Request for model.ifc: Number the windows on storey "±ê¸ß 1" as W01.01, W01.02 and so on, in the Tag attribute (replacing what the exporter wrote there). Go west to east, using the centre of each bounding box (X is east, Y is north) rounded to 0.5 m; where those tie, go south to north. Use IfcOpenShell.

First a look at what the model holds.

```python
import ifcopenshell
import ifcopenshell.util.element
import ifcopenshell.util.placement

model = ifcopenshell.open("model.ifc")
print(model.schema)
storey = next(s for s in model.by_type("IfcBuildingStorey") if s.Name == "±ê¸ß 1")
windows = [e for e in ifcopenshell.util.element.get_decomposition(storey) if e.is_a("IfcWindow")]
for e in sorted(windows, key=lambda e: e.id()):
    origin = ifcopenshell.util.placement.get_local_placement(e.ObjectPlacement)[:3, 3]
    print(e.id(), e.Tag, e.Name, origin.round(2) + 0.0, sep=" | ")
```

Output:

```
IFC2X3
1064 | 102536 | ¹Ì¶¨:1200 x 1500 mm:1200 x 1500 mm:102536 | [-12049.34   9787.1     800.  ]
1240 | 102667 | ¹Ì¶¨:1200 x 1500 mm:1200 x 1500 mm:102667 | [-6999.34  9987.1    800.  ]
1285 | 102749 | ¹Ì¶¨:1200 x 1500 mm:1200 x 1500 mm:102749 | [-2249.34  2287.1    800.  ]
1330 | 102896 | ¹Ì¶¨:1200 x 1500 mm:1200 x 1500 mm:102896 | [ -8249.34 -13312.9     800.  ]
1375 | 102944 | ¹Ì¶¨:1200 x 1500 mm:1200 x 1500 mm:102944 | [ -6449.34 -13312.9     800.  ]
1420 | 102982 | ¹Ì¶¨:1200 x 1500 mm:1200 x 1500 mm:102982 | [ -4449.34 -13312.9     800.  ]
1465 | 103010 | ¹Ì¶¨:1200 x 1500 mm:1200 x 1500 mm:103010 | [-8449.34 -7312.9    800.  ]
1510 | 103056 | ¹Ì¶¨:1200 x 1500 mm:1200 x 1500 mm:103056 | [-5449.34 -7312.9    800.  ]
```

```python
import ifcopenshell
import ifcopenshell.geom
import ifcopenshell.util.element
import ifcopenshell.util.shape

model = ifcopenshell.open("model.ifc")
settings = ifcopenshell.geom.settings()
settings.set("use-world-coords", True)


def centre(element):
    shape = ifcopenshell.geom.create_shape(settings, element)
    return ifcopenshell.util.shape.get_bbox_centroid(shape.geometry)


storey = next(s for s in model.by_type("IfcBuildingStorey") if s.Name == "±ê¸ß 1")
windows = [e for e in ifcopenshell.util.element.get_decomposition(storey) if e.is_a("IfcWindow")]

# Insertion points can sit at a corner or the storey origin, so sort by the geometry (in metres).
centres = {e: centre(e) for e in windows}
windows.sort(key=lambda e: (round(centres[e][0] / 0.5), centres[e][1]))

for i, e in enumerate(windows, start=1):
    number = f"W01.{i:02d}"
    e.Tag = number
    print(e.id(), number)

model.write("model_v2.ifc")
```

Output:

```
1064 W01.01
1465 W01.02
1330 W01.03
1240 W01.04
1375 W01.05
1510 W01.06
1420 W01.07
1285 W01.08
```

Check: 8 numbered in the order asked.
